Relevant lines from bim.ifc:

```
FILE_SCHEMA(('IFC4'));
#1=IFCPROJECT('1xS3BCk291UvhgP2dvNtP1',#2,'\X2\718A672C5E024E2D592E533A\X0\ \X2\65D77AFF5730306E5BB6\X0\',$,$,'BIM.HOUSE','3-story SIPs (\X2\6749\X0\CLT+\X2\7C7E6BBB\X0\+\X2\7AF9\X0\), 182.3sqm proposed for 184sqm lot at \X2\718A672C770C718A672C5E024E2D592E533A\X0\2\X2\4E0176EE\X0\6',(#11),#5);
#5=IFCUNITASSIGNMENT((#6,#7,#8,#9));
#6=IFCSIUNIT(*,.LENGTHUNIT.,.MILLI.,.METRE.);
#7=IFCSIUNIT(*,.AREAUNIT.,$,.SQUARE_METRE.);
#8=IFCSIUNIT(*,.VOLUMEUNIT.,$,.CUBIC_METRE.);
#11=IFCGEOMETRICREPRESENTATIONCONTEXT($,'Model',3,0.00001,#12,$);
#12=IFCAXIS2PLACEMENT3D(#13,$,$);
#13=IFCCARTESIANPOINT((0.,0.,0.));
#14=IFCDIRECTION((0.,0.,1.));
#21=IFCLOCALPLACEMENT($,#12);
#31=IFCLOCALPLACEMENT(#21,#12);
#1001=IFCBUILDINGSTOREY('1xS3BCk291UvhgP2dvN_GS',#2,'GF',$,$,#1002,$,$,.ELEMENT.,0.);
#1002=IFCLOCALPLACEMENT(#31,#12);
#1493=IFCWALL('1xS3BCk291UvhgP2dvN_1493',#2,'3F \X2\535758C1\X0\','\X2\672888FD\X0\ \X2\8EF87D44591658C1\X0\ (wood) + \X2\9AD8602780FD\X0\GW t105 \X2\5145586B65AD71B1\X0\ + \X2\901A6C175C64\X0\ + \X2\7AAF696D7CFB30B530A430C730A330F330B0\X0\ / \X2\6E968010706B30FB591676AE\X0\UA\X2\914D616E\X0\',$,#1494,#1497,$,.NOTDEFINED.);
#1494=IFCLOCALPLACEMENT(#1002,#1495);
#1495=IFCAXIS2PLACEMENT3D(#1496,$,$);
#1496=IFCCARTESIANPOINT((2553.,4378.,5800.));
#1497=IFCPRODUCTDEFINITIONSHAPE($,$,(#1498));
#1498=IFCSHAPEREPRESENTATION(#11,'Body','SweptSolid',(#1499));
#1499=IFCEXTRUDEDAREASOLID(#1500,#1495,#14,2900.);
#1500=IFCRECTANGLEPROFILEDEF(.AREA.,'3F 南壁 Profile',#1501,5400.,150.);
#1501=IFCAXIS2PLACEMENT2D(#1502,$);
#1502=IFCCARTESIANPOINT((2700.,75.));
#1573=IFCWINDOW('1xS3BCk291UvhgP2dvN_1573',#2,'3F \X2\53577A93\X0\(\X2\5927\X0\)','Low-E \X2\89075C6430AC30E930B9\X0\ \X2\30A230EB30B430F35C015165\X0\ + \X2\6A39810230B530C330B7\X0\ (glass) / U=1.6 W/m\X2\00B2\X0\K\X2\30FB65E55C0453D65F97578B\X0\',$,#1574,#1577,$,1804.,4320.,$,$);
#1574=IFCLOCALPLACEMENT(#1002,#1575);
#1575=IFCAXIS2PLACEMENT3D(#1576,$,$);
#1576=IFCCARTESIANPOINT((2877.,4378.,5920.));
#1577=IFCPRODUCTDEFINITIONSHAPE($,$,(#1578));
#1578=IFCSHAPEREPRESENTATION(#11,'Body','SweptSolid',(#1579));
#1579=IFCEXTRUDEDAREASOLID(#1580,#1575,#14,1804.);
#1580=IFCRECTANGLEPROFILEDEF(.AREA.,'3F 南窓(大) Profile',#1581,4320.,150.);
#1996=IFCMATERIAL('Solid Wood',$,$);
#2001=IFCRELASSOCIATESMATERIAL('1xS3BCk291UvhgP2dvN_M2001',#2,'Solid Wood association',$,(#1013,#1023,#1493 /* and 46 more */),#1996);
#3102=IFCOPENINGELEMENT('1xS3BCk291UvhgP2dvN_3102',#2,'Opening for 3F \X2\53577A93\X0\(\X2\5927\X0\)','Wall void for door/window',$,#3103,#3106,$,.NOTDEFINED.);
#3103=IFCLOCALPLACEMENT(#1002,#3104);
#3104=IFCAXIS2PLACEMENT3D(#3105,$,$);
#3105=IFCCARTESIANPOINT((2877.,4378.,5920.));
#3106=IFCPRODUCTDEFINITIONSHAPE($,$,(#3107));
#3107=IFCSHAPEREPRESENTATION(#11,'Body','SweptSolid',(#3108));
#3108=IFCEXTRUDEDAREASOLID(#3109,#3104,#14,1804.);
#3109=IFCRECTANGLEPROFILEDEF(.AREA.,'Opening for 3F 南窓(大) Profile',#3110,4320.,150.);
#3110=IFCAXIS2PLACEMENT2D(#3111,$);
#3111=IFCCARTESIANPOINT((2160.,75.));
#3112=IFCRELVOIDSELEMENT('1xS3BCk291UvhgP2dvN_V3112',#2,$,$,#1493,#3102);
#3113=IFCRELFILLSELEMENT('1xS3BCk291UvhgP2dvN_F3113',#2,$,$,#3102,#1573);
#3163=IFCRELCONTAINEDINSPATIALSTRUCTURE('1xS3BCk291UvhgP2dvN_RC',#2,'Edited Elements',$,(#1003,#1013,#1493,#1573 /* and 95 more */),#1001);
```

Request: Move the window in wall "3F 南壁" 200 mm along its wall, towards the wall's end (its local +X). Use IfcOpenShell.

```python
import ifcopenshell
import ifcopenshell.api.geometry
import ifcopenshell.util.placement
import ifcopenshell.util.unit

model = ifcopenshell.open("bim.ifc")
unit_scale = ifcopenshell.util.unit.calculate_unit_scale(model)

window = model.by_id(1573)
opening = window.FillsVoids[0].RelatingOpeningElement
wall = opening.VoidsElements[0].RelatingBuildingElement

wall_matrix = ifcopenshell.util.placement.get_local_placement(wall.ObjectPlacement)
shift = wall_matrix[:3, 0] * 0.2 / unit_scale
before = ifcopenshell.util.placement.get_local_placement(window.ObjectPlacement)[:3, 3].copy()

# The window is not placed relative to its opening, so move both.
for product in (opening, window):
    matrix = ifcopenshell.util.placement.get_local_placement(product.ObjectPlacement)
    matrix[:3, 3] += shift
    ifcopenshell.api.geometry.edit_object_placement(model, product=product, matrix=matrix, is_si=False)

after = ifcopenshell.util.placement.get_local_placement(window.ObjectPlacement)[:3, 3]
print("window moved by", (after - before).round(3) + 0.0)

model.write("bim_updated.ifc")
```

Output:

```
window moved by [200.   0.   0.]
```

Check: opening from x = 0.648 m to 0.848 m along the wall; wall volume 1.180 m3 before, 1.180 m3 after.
